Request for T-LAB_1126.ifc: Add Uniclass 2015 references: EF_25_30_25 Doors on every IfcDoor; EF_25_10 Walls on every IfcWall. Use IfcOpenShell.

First a look at what the model holds.

```python
import ifcopenshell

model = ifcopenshell.open("T-LAB_1126.ifc")
print(model.schema)
print("classifications:", [c.Name for c in model.by_type("IfcClassification")])
for ifc_class in ("IfcDoor", "IfcRoof", "IfcStair", "IfcWall", "IfcWindow"):
    print(ifc_class, len(model.by_type(ifc_class)))
```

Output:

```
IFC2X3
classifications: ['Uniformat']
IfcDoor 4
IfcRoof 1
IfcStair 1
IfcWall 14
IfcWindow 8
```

```python
import ifcopenshell
import ifcopenshell.api.classification

model = ifcopenshell.open("T-LAB_1126.ifc")

# IFC2X3 requires Source and Edition and has no link from the project to the system.
system = model.create_entity("IfcClassification", Source="NBS", Edition="2015", Name="Uniclass 2015")

codes = {
    "IfcDoor": ("EF_25_30_25", "Doors"),
    "IfcWall": ("EF_25_10", "Walls"),
}
for ifc_class, (code, name) in codes.items():
    products = model.by_type(ifc_class)
    ifcopenshell.api.classification.add_reference(
        model, products=products, classification=system, identification=code, name=name
    )
    print(code, len(products))

model.write("T-LAB_1126_rev.ifc")
```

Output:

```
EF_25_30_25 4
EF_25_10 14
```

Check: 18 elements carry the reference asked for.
